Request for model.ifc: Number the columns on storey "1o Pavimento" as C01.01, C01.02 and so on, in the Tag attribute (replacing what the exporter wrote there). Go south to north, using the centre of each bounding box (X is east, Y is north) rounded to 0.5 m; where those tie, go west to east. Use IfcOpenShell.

First a look at what the model holds.

```python
import ifcopenshell
import ifcopenshell.util.element
import ifcopenshell.util.placement

model = ifcopenshell.open("model.ifc")
print(model.schema)
storey = next(s for s in model.by_type("IfcBuildingStorey") if s.Name == "1o Pavimento")
columns = [e for e in ifcopenshell.util.element.get_decomposition(storey) if e.is_a("IfcColumn")]
for e in sorted(columns, key=lambda e: e.id()):
    origin = ifcopenshell.util.placement.get_local_placement(e.ObjectPlacement)[:3, 3]
    print(e.id(), e.Tag, e.Name, origin.round(2) + 0.0, sep=" | ")
```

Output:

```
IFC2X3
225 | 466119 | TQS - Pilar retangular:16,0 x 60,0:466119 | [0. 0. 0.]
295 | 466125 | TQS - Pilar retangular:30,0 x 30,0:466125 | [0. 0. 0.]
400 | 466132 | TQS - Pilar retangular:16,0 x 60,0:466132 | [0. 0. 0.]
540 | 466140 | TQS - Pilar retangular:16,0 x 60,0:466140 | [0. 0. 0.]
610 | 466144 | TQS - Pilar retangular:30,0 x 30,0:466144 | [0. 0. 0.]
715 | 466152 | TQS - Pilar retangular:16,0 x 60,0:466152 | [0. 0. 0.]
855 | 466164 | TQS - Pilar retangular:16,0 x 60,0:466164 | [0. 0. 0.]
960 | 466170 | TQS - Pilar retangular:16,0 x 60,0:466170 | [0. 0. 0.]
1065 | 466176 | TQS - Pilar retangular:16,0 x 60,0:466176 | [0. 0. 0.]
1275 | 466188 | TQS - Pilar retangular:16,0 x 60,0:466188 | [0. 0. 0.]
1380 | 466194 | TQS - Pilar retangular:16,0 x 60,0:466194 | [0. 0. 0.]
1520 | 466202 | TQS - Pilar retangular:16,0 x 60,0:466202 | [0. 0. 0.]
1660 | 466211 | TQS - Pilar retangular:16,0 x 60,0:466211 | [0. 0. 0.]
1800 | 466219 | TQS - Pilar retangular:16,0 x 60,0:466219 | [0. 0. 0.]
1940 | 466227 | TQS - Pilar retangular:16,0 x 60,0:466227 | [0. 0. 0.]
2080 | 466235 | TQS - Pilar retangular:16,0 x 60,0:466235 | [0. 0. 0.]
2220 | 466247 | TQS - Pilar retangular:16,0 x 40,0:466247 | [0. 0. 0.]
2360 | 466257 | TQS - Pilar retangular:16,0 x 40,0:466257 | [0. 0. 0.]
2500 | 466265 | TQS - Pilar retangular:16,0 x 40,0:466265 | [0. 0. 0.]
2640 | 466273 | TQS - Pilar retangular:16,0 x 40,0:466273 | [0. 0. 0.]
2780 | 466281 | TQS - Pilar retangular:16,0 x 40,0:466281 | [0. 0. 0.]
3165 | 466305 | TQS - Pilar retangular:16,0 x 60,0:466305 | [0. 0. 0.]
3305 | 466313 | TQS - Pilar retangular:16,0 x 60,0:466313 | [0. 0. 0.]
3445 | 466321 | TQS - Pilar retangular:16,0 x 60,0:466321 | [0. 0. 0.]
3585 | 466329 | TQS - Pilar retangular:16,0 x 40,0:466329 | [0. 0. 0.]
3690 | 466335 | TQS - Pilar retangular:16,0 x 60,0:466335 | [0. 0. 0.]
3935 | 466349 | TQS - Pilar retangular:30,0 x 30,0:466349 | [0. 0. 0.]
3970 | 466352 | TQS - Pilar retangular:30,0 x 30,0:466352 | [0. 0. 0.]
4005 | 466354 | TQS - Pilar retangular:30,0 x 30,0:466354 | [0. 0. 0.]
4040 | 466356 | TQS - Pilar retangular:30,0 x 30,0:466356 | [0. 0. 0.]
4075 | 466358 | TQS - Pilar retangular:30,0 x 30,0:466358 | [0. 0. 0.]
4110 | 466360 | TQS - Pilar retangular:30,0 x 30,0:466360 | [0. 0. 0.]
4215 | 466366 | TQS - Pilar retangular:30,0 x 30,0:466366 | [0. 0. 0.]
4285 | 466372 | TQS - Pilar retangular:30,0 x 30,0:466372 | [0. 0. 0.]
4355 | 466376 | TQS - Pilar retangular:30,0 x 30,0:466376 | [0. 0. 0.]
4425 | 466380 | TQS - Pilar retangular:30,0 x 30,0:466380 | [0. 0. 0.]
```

```python
import ifcopenshell
import ifcopenshell.geom
import ifcopenshell.util.element
import ifcopenshell.util.shape

model = ifcopenshell.open("model.ifc")
settings = ifcopenshell.geom.settings()
settings.set("use-world-coords", True)


def centre(element):
    shape = ifcopenshell.geom.create_shape(settings, element)
    return ifcopenshell.util.shape.get_bbox_centroid(shape.geometry)


storey = next(s for s in model.by_type("IfcBuildingStorey") if s.Name == "1o Pavimento")
columns = [e for e in ifcopenshell.util.element.get_decomposition(storey) if e.is_a("IfcColumn")]

# Insertion points can sit at a corner or the storey origin, so sort by the geometry (in metres).
centres = {e: centre(e) for e in columns}
columns.sort(key=lambda e: (round(centres[e][1] / 0.5), centres[e][0]))

for i, e in enumerate(columns, start=1):
    number = f"C01.{i:02d}"
    e.Tag = number
    print(e.id(), number)

model.write("model_edited.ifc")
```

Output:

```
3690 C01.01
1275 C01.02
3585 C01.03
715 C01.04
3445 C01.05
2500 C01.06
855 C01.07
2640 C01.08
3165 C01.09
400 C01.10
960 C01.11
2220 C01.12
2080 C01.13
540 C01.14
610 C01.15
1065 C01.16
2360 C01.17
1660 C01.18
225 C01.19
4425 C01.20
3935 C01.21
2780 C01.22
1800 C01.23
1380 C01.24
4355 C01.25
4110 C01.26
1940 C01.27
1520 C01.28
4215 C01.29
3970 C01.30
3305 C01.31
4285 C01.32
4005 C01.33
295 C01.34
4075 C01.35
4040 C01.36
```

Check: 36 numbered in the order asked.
